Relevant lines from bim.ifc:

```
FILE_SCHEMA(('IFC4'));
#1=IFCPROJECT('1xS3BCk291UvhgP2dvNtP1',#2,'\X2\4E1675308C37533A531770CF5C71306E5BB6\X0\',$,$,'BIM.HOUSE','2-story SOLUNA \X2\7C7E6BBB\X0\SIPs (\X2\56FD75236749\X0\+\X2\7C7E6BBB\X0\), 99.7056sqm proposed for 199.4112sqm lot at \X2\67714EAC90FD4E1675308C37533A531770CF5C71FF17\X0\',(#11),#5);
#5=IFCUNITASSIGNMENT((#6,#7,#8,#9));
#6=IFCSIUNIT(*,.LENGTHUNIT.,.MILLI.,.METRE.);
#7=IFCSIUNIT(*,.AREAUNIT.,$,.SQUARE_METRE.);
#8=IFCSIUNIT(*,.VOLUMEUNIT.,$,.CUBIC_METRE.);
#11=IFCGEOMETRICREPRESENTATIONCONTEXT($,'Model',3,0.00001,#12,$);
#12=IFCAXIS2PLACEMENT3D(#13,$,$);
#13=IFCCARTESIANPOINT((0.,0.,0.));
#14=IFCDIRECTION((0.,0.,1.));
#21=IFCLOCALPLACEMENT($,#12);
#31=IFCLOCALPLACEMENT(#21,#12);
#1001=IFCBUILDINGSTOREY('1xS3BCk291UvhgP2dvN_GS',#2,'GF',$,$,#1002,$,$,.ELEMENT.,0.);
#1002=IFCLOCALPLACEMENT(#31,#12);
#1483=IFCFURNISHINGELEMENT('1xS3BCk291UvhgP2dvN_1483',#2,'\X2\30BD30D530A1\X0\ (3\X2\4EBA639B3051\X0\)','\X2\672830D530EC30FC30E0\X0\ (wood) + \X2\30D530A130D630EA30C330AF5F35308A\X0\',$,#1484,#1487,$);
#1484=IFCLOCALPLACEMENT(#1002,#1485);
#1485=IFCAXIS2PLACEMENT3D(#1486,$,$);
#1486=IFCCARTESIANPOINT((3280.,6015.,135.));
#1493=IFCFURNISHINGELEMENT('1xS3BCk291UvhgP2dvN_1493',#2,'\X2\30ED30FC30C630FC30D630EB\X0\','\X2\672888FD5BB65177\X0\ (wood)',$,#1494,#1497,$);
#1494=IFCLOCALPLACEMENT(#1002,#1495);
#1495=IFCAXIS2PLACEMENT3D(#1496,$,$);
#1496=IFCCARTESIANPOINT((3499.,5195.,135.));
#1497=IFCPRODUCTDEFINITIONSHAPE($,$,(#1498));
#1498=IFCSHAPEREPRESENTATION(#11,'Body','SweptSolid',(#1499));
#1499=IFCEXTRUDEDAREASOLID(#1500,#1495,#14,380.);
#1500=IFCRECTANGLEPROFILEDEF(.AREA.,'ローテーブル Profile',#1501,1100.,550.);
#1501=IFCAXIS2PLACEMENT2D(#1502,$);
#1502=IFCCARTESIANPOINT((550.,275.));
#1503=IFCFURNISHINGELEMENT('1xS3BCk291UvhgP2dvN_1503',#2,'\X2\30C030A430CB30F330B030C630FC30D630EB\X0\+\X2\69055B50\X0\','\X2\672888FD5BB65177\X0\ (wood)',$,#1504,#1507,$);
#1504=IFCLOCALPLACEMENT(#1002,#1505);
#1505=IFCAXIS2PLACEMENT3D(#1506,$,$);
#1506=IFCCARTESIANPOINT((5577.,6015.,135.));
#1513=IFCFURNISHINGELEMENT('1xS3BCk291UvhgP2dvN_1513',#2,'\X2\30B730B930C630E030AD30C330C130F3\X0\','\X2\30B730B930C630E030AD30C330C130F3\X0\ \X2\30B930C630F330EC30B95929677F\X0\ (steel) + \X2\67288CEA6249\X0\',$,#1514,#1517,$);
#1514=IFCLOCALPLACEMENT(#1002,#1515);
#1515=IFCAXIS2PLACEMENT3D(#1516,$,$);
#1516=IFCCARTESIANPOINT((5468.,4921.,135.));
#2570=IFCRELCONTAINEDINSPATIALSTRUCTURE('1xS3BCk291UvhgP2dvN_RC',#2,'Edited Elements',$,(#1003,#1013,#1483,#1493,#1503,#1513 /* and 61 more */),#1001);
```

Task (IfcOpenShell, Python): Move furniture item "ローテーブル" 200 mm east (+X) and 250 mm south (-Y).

```python
import ifcopenshell
import ifcopenshell.api.geometry
import ifcopenshell.util.placement
import ifcopenshell.util.unit

model = ifcopenshell.open("bim.ifc")
unit_scale = ifcopenshell.util.unit.calculate_unit_scale(model)

item = model.by_guid("1xS3BCk291UvhgP2dvN_1493")
matrix = ifcopenshell.util.placement.get_local_placement(item.ObjectPlacement)
matrix[0, 3] += 0.2 / unit_scale
matrix[1, 3] -= 0.25 / unit_scale
ifcopenshell.api.geometry.edit_object_placement(model, product=item, matrix=matrix, is_si=False)

print(ifcopenshell.util.placement.get_local_placement(item.ObjectPlacement).round(3) + 0.0)

model.write("bim_updated.ifc")
```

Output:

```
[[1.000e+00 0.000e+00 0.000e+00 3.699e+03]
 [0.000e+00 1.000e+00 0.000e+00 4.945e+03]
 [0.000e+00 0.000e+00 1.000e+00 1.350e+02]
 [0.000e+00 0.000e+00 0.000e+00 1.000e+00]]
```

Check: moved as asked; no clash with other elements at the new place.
